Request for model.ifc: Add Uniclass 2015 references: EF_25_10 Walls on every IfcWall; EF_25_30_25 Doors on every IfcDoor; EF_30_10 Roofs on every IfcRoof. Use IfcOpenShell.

First a look at what the model holds.

```python
import ifcopenshell

model = ifcopenshell.open("model.ifc")
print(model.schema)
print("classifications:", [c.Name for c in model.by_type("IfcClassification")])
for ifc_class in ("IfcDoor", "IfcRoof", "IfcStair", "IfcWall", "IfcWindow"):
    print(ifc_class, len(model.by_type(ifc_class)))
```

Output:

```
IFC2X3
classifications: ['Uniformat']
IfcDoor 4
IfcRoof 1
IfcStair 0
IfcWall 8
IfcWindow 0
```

```python
import ifcopenshell
import ifcopenshell.api.classification

model = ifcopenshell.open("model.ifc")

# IFC2X3 requires Source and Edition and has no link from the project to the system.
system = model.create_entity("IfcClassification", Source="NBS", Edition="2015", Name="Uniclass 2015")

codes = {
    "IfcWall": ("EF_25_10", "Walls"),
    "IfcDoor": ("EF_25_30_25", "Doors"),
    "IfcRoof": ("EF_30_10", "Roofs"),
}
for ifc_class, (code, name) in codes.items():
    products = model.by_type(ifc_class)
    ifcopenshell.api.classification.add_reference(
        model, products=products, classification=system, identification=code, name=name
    )
    print(code, len(products))

model.write("model_updated.ifc")
```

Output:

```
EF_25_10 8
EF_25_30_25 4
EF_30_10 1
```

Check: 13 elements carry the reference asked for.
